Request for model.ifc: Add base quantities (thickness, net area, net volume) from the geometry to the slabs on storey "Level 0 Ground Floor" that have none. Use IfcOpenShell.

First a look at what the model holds.

```python
import ifcopenshell
import ifcopenshell.util.element
import ifcopenshell.util.unit

model = ifcopenshell.open("model.ifc")
print(model.schema)
for unit_type in ("LENGTHUNIT", "AREAUNIT", "VOLUMEUNIT"):
    print(unit_type, ifcopenshell.util.unit.calculate_unit_scale(model, unit_type))
storey = next(s for s in model.by_type("IfcBuildingStorey") if s.Name == "Level 0 Ground Floor")
slabs = [e for e in ifcopenshell.util.element.get_decomposition(storey) if e.is_a("IfcSlab")]
for e in sorted(slabs, key=lambda e: e.id()):
    print(e.id(), e.is_a(), e.Name, list(ifcopenshell.util.element.get_psets(e, qtos_only=True)), sep=" | ")
```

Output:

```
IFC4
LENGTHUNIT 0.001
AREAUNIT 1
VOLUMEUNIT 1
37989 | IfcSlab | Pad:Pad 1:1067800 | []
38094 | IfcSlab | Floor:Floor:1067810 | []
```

```python
import ifcopenshell
import ifcopenshell.api.pset
import ifcopenshell.geom
import ifcopenshell.util.element
import ifcopenshell.util.shape
import ifcopenshell.util.unit

model = ifcopenshell.open("model.ifc")
unit_scale = ifcopenshell.util.unit.calculate_unit_scale(model)
area_scale = ifcopenshell.util.unit.calculate_unit_scale(model, "AREAUNIT")
volume_scale = ifcopenshell.util.unit.calculate_unit_scale(model, "VOLUMEUNIT")
settings = ifcopenshell.geom.settings()

storey = next(s for s in model.by_type("IfcBuildingStorey") if s.Name == "Level 0 Ground Floor")
slabs = [e for e in ifcopenshell.util.element.get_decomposition(storey) if e.is_a("IfcSlab")]

for e in sorted(slabs, key=lambda e: e.id()):
    if ifcopenshell.util.element.get_psets(e, qtos_only=True, should_inherit=False):
        continue
    # Geometry comes back in metres, in the element's own axes.
    shape = ifcopenshell.geom.create_shape(settings, e)
    values = {
        "Width": ifcopenshell.util.shape.get_z(shape.geometry) / unit_scale,
        "NetArea": ifcopenshell.util.shape.get_footprint_area(shape.geometry) / area_scale,
        "NetVolume": ifcopenshell.util.shape.get_volume(shape.geometry) / volume_scale,
    }
    qto = ifcopenshell.api.pset.add_qto(model, product=e, name="Qto_SlabBaseQuantities")
    ifcopenshell.api.pset.edit_qto(model, qto=qto, properties=values)
    print(e.id(), {k: round(v, 3) for k, v in values.items()})

model.write("model_v2.ifc")
```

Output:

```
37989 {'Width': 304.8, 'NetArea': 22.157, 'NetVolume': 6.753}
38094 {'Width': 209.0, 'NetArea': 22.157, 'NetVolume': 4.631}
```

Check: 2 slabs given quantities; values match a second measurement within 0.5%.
